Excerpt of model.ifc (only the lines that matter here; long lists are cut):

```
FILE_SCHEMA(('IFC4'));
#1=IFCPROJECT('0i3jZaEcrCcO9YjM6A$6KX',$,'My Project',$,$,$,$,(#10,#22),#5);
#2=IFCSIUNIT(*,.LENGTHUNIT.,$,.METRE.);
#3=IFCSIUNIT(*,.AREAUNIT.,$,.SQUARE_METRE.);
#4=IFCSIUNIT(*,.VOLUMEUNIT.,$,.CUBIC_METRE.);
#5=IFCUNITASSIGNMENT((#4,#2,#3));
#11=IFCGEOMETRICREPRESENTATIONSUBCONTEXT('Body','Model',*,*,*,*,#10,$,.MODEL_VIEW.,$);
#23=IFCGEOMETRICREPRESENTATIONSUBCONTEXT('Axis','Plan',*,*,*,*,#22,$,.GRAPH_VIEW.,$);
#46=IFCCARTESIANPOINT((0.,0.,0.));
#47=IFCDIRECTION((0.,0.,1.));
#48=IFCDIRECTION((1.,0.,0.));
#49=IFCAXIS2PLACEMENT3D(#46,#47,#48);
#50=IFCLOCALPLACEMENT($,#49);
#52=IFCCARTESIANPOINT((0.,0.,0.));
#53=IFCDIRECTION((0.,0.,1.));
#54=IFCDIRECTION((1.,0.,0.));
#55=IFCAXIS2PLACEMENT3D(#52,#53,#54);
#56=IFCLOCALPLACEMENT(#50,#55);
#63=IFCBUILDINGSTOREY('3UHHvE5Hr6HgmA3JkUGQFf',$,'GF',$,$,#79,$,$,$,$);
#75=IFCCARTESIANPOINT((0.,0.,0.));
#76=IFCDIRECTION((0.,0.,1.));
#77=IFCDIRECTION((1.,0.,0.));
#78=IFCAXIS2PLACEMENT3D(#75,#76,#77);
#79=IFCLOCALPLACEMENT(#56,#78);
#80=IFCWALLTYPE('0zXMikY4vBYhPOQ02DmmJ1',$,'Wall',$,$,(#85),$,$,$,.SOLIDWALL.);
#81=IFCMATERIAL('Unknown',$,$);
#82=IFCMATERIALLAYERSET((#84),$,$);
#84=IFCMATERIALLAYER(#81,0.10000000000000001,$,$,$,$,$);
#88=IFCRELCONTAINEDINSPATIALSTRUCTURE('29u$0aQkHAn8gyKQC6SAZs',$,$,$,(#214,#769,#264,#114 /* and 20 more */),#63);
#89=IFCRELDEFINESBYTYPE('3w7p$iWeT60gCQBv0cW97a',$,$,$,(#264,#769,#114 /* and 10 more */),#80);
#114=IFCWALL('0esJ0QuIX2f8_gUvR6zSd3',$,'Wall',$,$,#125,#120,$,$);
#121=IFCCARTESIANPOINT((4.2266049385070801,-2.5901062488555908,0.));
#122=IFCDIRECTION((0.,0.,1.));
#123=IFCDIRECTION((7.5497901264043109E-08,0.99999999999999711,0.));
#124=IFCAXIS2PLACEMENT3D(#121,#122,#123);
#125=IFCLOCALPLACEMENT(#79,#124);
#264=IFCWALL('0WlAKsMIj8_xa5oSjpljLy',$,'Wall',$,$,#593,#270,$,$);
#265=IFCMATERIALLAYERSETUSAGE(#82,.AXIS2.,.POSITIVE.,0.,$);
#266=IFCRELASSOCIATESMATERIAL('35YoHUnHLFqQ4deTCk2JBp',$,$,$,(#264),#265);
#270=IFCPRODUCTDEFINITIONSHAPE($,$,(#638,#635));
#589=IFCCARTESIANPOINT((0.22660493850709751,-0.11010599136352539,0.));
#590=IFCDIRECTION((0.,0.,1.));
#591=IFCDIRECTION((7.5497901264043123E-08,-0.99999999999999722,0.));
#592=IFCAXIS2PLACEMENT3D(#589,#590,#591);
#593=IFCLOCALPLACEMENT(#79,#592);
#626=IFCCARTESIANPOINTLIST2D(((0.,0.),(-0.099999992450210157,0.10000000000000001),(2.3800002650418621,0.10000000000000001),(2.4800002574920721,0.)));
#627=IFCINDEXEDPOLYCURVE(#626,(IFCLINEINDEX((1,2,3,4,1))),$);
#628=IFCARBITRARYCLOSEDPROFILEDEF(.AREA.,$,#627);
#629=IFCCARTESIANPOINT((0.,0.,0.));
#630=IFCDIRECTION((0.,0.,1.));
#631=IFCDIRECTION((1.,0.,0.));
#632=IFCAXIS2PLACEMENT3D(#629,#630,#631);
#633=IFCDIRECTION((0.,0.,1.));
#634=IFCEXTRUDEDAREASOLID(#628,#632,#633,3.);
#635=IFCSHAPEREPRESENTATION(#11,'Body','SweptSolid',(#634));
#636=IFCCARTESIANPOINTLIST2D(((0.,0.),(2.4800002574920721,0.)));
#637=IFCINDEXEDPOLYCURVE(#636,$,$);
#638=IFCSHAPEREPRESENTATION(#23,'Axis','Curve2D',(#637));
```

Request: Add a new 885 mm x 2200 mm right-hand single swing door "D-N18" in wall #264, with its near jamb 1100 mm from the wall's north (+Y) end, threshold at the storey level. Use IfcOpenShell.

```python
import numpy as np
import ifcopenshell
import ifcopenshell.api.feature
import ifcopenshell.api.geometry
import ifcopenshell.api.root
import ifcopenshell.api.spatial
import ifcopenshell.geom
import ifcopenshell.util.element
import ifcopenshell.util.placement
import ifcopenshell.util.representation
import ifcopenshell.util.shape
import ifcopenshell.util.unit

model = ifcopenshell.open("model.ifc")
unit_scale = ifcopenshell.util.unit.calculate_unit_scale(model)
settings = ifcopenshell.geom.settings()


def volume(element):
    """Net volume in cubic metres, openings subtracted."""
    shape = ifcopenshell.geom.create_shape(settings, element)
    return ifcopenshell.util.shape.get_volume(shape.geometry)


wall = model.by_id(264)
storey = ifcopenshell.util.element.get_container(wall, ifc_class="IfcBuildingStorey")
context = ifcopenshell.util.representation.get_context(model, "Model", "Body", "MODEL_VIEW")
before = volume(wall)

width, height, from_end, sill = 0.885, 2.2, 1.1, 0.0  # metres

# The wall runs along its own X axis, and the end named is its -X end.
wall_shape = ifcopenshell.geom.create_shape(settings, wall)
x, y, z = ifcopenshell.util.shape.get_vertices(wall_shape.geometry).T
start = x.min() + from_end
face, thickness = float(y.min()), float(y.max() - y.min())
wall_matrix = ifcopenshell.util.placement.get_local_placement(wall.ObjectPlacement)
level = ifcopenshell.util.placement.get_local_placement(storey.ObjectPlacement)[2, 3]


def in_wall(x, y):
    """Placement at x, y metres in the wall's axes, at sill height."""
    matrix = wall_matrix.copy()
    matrix[:, 3] = wall_matrix @ np.array([x / unit_scale, y / unit_scale, 0.0, 1.0])
    matrix[2, 3] = level + sill / unit_scale
    return matrix


# Opening: a box that overshoots both wall faces by 50 mm.
opening = ifcopenshell.api.root.create_entity(model, ifc_class="IfcOpeningElement", predefined_type="OPENING")
box = ifcopenshell.api.geometry.add_wall_representation(
    model, context=context, length=width, height=height, thickness=thickness + 0.1
)
ifcopenshell.api.geometry.assign_representation(model, product=opening, representation=box)
ifcopenshell.api.geometry.edit_object_placement(model, product=opening, matrix=in_wall(start, face - 0.05), is_si=False)
ifcopenshell.api.feature.add_feature(model, feature=opening, element=wall)

door = ifcopenshell.api.root.create_entity(model, ifc_class="IfcDoor", name="D-N18", predefined_type="DOOR")
door.OverallWidth, door.OverallHeight = width / unit_scale, height / unit_scale
door.OperationType = "SINGLE_SWING_RIGHT"
body = ifcopenshell.api.geometry.add_door_representation(
    model,
    context=context,
    overall_width=door.OverallWidth,
    overall_height=door.OverallHeight,
    operation_type="SINGLE_SWING_RIGHT",
    lining_properties={"LiningDepth": thickness / unit_scale, "ThresholdDepth": thickness / unit_scale},
)
ifcopenshell.api.geometry.assign_representation(model, product=door, representation=body)
ifcopenshell.api.spatial.assign_container(model, products=[door], relating_structure=storey)
ifcopenshell.api.feature.add_filling(model, opening=opening, element=door)

# The lining spans the wall, so the door starts at the wall face.
ifcopenshell.api.geometry.edit_object_placement(model, product=door, matrix=in_wall(start, face), is_si=False)

after = volume(wall)

print(f"wall volume {before:.3f} -> {after:.3f} m3")

model.write("model_updated.ifc")
```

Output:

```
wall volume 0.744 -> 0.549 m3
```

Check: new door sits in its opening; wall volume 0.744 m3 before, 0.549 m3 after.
